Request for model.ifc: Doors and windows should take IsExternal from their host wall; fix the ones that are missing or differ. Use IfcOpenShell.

First a look at what the model holds.

```python
import ifcopenshell
import ifcopenshell.util.element

model = ifcopenshell.open("model.ifc")
print(model.schema)
seen = {}
for e in model.by_type("IfcDoor") + model.by_type("IfcWindow"):
    if not e.FillsVoids:
        continue
    host = e.FillsVoids[0].RelatingOpeningElement.VoidsElements[0].RelatingBuildingElement
    own = ifcopenshell.util.element.get_pset(e, f"Pset_{e.is_a()[3:].removesuffix('StandardCase')}Common", "IsExternal")
    wall = ifcopenshell.util.element.get_pset(host, "Pset_WallCommon", "IsExternal")
    seen[e.is_a(), own, wall] = seen.get((e.is_a(), own, wall), 0) + 1
for (cls, own, wall), count in sorted(seen.items(), key=str):
    print(count, cls, "IsExternal:", own, "| host wall:", wall)
```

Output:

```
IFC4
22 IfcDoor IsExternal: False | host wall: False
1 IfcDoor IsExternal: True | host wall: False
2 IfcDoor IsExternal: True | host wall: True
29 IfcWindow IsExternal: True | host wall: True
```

```python
import ifcopenshell
import ifcopenshell.api.pset
import ifcopenshell.util.element

model = ifcopenshell.open("model.ifc")

count = 0
for ifc_class, pset_name in (("IfcDoor", "Pset_DoorCommon"), ("IfcWindow", "Pset_WindowCommon")):
    for e in model.by_type(ifc_class):
        if not e.FillsVoids:
            continue
        host = e.FillsVoids[0].RelatingOpeningElement.VoidsElements[0].RelatingBuildingElement
        external = ifcopenshell.util.element.get_pset(host, "Pset_WallCommon", "IsExternal")
        if external is None or ifcopenshell.util.element.get_pset(e, pset_name, "IsExternal") == external:
            continue
        pset = ifcopenshell.api.pset.add_pset(model, product=e, name=pset_name)
        ifcopenshell.api.pset.edit_pset(model, pset=pset, properties={"IsExternal": external})
        count += 1

print(count, "updated")

model.write("model_v2.ifc")
```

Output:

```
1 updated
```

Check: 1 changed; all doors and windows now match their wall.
